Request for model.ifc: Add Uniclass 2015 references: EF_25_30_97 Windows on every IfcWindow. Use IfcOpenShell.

First a look at what the model holds.

```python
import ifcopenshell

model = ifcopenshell.open("model.ifc")
print(model.schema)
print("classifications:", [c.Name for c in model.by_type("IfcClassification")])
for ifc_class in ("IfcDoor", "IfcRoof", "IfcStair", "IfcWall", "IfcWindow"):
    print(ifc_class, len(model.by_type(ifc_class)))
```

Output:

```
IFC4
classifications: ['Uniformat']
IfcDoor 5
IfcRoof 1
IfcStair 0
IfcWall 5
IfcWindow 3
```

```python
import ifcopenshell
import ifcopenshell.api.classification

model = ifcopenshell.open("model.ifc")

system = ifcopenshell.api.classification.add_classification(model, classification="Uniclass 2015")

codes = {
    "IfcWindow": ("EF_25_30_97", "Windows"),
}
for ifc_class, (code, name) in codes.items():
    products = model.by_type(ifc_class)
    ifcopenshell.api.classification.add_reference(
        model, products=products, classification=system, identification=code, name=name
    )
    print(code, len(products))

model.write("model_edited.ifc")
```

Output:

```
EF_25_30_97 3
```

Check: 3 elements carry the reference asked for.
